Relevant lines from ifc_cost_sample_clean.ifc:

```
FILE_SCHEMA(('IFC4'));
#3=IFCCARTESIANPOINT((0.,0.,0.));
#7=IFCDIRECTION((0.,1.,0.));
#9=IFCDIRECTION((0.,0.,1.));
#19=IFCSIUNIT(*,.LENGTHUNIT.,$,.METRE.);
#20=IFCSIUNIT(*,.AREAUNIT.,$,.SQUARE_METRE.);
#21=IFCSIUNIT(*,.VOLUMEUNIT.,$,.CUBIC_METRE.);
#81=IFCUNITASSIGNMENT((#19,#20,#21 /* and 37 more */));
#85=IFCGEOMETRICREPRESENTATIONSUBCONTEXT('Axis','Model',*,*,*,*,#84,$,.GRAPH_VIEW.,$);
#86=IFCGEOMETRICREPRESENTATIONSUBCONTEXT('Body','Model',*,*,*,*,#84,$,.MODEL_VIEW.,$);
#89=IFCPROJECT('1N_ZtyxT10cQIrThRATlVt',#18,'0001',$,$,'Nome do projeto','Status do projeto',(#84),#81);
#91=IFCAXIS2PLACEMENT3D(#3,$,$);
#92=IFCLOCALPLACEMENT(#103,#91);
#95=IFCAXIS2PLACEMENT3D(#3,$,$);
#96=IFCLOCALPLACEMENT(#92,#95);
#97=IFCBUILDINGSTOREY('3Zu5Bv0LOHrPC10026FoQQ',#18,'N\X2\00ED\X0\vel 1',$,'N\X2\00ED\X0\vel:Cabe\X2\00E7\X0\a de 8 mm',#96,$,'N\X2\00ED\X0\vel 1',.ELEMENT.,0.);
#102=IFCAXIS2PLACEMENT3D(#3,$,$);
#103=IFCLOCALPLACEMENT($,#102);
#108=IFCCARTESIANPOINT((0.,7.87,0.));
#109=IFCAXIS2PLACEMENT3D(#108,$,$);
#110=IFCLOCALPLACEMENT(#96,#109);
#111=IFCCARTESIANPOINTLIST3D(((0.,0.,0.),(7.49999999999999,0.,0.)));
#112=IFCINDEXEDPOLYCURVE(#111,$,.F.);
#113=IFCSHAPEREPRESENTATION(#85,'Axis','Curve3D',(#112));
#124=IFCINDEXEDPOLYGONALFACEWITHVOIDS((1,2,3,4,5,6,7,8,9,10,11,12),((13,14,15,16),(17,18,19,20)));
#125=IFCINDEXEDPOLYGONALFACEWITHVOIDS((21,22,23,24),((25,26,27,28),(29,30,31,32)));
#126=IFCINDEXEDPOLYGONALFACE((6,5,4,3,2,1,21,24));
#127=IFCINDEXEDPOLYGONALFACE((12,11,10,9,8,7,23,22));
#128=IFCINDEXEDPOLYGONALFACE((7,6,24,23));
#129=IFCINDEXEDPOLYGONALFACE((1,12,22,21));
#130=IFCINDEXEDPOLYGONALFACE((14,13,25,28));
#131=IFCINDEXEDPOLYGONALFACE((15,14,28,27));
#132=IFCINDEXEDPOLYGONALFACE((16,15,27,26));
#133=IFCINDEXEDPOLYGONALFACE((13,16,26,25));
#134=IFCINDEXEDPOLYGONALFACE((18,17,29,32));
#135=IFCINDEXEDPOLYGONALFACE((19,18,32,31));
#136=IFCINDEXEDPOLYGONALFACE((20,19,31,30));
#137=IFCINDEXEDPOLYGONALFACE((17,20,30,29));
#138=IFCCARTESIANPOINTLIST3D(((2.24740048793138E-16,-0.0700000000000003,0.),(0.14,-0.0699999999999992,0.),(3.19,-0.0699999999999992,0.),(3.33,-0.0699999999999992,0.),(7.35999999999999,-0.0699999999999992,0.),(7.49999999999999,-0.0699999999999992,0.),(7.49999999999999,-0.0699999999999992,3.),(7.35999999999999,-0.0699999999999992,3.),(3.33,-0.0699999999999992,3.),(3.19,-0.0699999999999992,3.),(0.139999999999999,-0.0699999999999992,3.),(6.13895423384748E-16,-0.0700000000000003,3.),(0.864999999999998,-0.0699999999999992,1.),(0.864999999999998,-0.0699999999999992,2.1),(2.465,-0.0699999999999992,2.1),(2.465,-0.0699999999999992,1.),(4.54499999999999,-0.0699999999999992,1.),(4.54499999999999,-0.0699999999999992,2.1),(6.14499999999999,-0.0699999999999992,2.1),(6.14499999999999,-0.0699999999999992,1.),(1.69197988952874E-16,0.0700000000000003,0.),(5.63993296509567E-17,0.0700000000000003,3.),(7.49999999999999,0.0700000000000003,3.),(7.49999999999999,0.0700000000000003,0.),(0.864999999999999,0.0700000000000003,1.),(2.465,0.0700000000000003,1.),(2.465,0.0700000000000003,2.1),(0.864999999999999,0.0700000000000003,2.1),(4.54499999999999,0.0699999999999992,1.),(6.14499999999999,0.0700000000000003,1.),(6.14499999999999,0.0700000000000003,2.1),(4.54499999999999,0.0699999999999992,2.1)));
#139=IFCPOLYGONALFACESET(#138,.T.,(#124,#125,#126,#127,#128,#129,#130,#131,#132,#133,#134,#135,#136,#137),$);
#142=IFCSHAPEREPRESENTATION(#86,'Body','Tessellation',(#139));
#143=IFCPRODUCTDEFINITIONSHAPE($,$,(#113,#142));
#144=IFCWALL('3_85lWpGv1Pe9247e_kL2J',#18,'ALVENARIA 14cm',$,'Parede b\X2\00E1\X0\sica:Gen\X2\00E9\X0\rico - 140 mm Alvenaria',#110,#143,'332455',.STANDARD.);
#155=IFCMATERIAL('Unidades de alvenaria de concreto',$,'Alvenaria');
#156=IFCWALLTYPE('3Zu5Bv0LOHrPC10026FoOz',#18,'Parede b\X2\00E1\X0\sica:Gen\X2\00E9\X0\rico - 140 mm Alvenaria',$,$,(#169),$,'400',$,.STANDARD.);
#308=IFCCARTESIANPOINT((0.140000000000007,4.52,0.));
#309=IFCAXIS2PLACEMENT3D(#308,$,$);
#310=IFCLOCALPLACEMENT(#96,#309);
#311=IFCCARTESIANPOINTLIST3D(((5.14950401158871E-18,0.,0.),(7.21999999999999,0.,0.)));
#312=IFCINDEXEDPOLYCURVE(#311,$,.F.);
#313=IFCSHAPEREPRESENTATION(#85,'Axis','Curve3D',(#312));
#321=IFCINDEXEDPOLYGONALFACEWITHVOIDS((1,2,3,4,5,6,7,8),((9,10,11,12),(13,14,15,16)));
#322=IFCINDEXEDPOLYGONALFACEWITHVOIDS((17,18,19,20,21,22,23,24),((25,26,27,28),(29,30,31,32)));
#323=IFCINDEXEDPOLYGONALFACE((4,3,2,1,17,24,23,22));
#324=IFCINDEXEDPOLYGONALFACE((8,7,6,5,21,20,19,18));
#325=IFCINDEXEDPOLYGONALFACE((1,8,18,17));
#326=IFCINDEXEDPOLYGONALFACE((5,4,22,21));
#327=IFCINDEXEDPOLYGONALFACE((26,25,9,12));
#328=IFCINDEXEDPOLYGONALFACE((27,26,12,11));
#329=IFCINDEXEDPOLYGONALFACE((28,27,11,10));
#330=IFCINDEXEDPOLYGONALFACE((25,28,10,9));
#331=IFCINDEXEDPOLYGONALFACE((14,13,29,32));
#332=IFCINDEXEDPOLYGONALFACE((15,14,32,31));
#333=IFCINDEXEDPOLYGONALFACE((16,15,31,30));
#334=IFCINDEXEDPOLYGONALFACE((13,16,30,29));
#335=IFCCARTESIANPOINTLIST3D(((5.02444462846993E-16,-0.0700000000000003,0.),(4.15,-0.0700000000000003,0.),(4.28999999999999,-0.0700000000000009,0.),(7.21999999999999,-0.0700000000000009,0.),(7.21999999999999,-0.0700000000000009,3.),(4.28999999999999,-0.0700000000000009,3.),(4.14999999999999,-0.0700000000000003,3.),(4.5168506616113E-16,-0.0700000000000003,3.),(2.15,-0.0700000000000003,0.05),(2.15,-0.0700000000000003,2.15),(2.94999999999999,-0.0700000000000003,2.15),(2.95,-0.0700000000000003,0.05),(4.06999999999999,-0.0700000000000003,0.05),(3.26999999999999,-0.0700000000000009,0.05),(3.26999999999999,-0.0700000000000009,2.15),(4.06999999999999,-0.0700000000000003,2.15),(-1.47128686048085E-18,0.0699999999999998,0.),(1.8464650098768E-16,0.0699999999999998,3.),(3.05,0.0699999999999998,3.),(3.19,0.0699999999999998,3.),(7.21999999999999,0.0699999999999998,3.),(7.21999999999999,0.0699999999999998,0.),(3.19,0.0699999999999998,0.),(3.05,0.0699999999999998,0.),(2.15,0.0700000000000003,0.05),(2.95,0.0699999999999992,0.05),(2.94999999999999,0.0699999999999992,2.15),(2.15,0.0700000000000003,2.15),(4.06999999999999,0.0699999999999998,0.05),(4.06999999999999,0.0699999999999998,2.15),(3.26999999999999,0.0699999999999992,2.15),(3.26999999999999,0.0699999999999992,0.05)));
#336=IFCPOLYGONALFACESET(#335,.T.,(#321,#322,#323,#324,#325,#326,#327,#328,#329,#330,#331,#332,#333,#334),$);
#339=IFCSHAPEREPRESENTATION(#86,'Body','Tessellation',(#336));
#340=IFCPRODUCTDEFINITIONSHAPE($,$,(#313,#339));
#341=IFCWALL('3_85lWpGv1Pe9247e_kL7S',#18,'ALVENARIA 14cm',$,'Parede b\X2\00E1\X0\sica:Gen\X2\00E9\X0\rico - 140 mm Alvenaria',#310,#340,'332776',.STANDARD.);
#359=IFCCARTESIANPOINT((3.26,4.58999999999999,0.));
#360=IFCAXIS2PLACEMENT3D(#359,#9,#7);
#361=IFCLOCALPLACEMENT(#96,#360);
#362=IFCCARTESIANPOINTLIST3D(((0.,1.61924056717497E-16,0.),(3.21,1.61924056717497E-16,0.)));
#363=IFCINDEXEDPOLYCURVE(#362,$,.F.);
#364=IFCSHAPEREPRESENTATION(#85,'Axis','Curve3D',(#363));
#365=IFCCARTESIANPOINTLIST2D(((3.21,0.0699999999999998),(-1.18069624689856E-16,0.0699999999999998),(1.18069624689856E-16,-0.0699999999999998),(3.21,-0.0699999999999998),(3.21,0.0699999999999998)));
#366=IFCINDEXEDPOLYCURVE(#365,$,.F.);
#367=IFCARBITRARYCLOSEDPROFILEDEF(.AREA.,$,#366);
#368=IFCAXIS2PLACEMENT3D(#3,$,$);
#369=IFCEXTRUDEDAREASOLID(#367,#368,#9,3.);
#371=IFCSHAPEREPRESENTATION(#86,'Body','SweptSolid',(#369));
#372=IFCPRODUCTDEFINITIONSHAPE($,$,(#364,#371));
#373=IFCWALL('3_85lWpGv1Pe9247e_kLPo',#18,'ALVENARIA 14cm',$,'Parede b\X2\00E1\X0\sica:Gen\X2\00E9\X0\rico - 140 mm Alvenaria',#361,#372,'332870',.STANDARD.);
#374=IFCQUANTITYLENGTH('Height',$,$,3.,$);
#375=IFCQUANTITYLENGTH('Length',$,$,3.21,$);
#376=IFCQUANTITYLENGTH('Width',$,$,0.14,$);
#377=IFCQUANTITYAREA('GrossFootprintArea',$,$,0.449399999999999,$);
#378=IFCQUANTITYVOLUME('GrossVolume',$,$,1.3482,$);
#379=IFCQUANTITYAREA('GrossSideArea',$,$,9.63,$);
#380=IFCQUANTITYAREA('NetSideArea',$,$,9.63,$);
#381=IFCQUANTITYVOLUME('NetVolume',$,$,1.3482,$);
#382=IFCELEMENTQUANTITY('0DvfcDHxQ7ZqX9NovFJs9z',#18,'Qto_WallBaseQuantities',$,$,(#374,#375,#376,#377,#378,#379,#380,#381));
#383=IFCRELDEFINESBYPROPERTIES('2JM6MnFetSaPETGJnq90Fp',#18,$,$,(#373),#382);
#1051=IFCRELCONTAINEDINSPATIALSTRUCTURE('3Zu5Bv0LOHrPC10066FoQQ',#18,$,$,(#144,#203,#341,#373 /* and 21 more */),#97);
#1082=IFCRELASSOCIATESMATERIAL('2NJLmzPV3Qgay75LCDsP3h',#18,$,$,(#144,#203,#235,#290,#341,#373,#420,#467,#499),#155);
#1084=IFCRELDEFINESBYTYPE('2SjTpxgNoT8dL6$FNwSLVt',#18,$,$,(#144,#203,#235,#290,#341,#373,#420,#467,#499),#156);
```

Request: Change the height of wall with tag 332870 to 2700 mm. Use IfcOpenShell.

```python
import ifcopenshell
import ifcopenshell.api.pset
import ifcopenshell.geom
import ifcopenshell.util.element
import ifcopenshell.util.representation
import ifcopenshell.util.shape
import ifcopenshell.util.unit

model = ifcopenshell.open("ifc_cost_sample_clean.ifc")
unit_scale = ifcopenshell.util.unit.calculate_unit_scale(model)
area_scale = ifcopenshell.util.unit.calculate_unit_scale(model, "AREAUNIT")
volume_scale = ifcopenshell.util.unit.calculate_unit_scale(model, "VOLUMEUNIT")
settings = ifcopenshell.geom.settings()


def volume(element):
    """Net volume in cubic metres, openings subtracted."""
    shape = ifcopenshell.geom.create_shape(settings, element)
    return ifcopenshell.util.shape.get_volume(shape.geometry)


wall = model.by_guid("3_85lWpGv1Pe9247e_kLPo")
before = volume(wall)

body = ifcopenshell.util.representation.get_representation(wall, "Model", "Body")
solid = body.Items[0]
old_height = solid.Depth
solid.Depth = 2.7
after = volume(wall)
thickness = 0.14  # wall thickness in metres

# Update the stored height, areas and volumes.
qto = model.by_id(ifcopenshell.util.element.get_pset(wall, "Qto_WallBaseQuantities", should_inherit=False)["id"])
ifcopenshell.api.pset.edit_qto(model, qto=qto, properties={
    "Height": solid.Depth,
    "GrossVolume": ifcopenshell.util.element.get_pset(wall, "Qto_WallBaseQuantities", "GrossVolume") * solid.Depth / old_height,
    "GrossSideArea": ifcopenshell.util.element.get_pset(wall, "Qto_WallBaseQuantities", "GrossSideArea") * solid.Depth / old_height,
    "NetSideArea": after / thickness / area_scale,
    "NetVolume": after / volume_scale,
})

print(f"height {old_height:g} -> {solid.Depth:g}, volume {before:.3f} -> {after:.3f} m3")

model.write("ifc_cost_sample_clean-out.ifc")
```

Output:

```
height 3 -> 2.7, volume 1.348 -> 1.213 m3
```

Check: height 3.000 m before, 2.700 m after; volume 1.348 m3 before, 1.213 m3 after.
